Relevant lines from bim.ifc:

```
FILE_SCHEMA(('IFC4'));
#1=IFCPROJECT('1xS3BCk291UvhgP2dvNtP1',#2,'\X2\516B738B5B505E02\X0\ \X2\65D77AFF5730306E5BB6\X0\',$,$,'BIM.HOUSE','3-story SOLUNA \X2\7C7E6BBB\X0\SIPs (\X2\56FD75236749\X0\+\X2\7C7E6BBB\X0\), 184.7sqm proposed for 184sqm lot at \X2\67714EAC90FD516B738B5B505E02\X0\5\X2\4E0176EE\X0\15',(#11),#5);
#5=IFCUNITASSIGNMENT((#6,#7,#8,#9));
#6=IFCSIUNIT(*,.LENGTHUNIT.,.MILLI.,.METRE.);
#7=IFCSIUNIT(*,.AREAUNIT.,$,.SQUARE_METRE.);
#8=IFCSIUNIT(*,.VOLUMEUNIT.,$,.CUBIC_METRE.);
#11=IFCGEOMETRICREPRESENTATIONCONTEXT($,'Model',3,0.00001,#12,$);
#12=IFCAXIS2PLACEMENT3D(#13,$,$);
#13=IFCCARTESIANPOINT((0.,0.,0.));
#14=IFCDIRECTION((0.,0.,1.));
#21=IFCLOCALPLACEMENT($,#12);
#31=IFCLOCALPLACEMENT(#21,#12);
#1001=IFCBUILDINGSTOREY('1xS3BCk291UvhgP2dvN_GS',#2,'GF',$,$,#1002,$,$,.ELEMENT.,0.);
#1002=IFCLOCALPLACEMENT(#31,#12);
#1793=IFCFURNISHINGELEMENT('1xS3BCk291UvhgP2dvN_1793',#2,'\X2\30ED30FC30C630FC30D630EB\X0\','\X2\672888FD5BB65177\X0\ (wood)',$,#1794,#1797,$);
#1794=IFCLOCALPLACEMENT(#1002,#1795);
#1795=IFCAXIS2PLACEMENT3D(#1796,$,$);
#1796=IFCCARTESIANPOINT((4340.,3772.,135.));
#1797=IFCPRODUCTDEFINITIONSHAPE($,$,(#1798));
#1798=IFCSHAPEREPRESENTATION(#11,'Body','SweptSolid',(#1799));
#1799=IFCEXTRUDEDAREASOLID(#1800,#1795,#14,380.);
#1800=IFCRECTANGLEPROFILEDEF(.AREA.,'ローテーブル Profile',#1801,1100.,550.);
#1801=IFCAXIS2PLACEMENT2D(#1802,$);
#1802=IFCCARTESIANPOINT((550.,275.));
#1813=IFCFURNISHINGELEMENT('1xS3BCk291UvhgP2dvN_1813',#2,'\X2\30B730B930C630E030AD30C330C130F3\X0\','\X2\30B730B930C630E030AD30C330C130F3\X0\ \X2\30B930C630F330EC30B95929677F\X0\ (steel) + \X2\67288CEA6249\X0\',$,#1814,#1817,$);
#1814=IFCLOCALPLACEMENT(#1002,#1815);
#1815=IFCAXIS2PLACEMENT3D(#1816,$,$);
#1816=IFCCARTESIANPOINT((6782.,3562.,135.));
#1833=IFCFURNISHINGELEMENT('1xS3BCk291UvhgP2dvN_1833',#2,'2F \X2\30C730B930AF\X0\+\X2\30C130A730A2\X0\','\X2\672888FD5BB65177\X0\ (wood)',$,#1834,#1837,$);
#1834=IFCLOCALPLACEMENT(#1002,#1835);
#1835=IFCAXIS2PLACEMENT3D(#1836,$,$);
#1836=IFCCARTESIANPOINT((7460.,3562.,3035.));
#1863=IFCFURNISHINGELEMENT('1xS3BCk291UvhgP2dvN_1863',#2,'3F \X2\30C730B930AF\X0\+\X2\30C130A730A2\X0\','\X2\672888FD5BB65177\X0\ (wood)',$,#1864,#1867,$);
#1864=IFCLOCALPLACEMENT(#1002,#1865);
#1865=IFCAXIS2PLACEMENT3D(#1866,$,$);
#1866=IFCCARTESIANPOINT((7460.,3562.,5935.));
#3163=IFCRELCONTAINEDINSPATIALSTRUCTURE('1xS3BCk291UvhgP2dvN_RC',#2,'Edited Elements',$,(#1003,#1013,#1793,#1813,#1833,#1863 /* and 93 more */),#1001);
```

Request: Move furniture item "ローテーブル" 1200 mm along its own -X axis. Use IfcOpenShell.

```python
import ifcopenshell
import ifcopenshell.api.geometry
import ifcopenshell.util.placement
import ifcopenshell.util.unit

model = ifcopenshell.open("bim.ifc")
unit_scale = ifcopenshell.util.unit.calculate_unit_scale(model)

item = model.by_guid("1xS3BCk291UvhgP2dvN_1793")
matrix = ifcopenshell.util.placement.get_local_placement(item.ObjectPlacement)
matrix[:3, 3] -= matrix[:3, 0] * 1.2 / unit_scale
ifcopenshell.api.geometry.edit_object_placement(model, product=item, matrix=matrix, is_si=False)

print(ifcopenshell.util.placement.get_local_placement(item.ObjectPlacement).round(3) + 0.0)

model.write("bim_updated.ifc")
```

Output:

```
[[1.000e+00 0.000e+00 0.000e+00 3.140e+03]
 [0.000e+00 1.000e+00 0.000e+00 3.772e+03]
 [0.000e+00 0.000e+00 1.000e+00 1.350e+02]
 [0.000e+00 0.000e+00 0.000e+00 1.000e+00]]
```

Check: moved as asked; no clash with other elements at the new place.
